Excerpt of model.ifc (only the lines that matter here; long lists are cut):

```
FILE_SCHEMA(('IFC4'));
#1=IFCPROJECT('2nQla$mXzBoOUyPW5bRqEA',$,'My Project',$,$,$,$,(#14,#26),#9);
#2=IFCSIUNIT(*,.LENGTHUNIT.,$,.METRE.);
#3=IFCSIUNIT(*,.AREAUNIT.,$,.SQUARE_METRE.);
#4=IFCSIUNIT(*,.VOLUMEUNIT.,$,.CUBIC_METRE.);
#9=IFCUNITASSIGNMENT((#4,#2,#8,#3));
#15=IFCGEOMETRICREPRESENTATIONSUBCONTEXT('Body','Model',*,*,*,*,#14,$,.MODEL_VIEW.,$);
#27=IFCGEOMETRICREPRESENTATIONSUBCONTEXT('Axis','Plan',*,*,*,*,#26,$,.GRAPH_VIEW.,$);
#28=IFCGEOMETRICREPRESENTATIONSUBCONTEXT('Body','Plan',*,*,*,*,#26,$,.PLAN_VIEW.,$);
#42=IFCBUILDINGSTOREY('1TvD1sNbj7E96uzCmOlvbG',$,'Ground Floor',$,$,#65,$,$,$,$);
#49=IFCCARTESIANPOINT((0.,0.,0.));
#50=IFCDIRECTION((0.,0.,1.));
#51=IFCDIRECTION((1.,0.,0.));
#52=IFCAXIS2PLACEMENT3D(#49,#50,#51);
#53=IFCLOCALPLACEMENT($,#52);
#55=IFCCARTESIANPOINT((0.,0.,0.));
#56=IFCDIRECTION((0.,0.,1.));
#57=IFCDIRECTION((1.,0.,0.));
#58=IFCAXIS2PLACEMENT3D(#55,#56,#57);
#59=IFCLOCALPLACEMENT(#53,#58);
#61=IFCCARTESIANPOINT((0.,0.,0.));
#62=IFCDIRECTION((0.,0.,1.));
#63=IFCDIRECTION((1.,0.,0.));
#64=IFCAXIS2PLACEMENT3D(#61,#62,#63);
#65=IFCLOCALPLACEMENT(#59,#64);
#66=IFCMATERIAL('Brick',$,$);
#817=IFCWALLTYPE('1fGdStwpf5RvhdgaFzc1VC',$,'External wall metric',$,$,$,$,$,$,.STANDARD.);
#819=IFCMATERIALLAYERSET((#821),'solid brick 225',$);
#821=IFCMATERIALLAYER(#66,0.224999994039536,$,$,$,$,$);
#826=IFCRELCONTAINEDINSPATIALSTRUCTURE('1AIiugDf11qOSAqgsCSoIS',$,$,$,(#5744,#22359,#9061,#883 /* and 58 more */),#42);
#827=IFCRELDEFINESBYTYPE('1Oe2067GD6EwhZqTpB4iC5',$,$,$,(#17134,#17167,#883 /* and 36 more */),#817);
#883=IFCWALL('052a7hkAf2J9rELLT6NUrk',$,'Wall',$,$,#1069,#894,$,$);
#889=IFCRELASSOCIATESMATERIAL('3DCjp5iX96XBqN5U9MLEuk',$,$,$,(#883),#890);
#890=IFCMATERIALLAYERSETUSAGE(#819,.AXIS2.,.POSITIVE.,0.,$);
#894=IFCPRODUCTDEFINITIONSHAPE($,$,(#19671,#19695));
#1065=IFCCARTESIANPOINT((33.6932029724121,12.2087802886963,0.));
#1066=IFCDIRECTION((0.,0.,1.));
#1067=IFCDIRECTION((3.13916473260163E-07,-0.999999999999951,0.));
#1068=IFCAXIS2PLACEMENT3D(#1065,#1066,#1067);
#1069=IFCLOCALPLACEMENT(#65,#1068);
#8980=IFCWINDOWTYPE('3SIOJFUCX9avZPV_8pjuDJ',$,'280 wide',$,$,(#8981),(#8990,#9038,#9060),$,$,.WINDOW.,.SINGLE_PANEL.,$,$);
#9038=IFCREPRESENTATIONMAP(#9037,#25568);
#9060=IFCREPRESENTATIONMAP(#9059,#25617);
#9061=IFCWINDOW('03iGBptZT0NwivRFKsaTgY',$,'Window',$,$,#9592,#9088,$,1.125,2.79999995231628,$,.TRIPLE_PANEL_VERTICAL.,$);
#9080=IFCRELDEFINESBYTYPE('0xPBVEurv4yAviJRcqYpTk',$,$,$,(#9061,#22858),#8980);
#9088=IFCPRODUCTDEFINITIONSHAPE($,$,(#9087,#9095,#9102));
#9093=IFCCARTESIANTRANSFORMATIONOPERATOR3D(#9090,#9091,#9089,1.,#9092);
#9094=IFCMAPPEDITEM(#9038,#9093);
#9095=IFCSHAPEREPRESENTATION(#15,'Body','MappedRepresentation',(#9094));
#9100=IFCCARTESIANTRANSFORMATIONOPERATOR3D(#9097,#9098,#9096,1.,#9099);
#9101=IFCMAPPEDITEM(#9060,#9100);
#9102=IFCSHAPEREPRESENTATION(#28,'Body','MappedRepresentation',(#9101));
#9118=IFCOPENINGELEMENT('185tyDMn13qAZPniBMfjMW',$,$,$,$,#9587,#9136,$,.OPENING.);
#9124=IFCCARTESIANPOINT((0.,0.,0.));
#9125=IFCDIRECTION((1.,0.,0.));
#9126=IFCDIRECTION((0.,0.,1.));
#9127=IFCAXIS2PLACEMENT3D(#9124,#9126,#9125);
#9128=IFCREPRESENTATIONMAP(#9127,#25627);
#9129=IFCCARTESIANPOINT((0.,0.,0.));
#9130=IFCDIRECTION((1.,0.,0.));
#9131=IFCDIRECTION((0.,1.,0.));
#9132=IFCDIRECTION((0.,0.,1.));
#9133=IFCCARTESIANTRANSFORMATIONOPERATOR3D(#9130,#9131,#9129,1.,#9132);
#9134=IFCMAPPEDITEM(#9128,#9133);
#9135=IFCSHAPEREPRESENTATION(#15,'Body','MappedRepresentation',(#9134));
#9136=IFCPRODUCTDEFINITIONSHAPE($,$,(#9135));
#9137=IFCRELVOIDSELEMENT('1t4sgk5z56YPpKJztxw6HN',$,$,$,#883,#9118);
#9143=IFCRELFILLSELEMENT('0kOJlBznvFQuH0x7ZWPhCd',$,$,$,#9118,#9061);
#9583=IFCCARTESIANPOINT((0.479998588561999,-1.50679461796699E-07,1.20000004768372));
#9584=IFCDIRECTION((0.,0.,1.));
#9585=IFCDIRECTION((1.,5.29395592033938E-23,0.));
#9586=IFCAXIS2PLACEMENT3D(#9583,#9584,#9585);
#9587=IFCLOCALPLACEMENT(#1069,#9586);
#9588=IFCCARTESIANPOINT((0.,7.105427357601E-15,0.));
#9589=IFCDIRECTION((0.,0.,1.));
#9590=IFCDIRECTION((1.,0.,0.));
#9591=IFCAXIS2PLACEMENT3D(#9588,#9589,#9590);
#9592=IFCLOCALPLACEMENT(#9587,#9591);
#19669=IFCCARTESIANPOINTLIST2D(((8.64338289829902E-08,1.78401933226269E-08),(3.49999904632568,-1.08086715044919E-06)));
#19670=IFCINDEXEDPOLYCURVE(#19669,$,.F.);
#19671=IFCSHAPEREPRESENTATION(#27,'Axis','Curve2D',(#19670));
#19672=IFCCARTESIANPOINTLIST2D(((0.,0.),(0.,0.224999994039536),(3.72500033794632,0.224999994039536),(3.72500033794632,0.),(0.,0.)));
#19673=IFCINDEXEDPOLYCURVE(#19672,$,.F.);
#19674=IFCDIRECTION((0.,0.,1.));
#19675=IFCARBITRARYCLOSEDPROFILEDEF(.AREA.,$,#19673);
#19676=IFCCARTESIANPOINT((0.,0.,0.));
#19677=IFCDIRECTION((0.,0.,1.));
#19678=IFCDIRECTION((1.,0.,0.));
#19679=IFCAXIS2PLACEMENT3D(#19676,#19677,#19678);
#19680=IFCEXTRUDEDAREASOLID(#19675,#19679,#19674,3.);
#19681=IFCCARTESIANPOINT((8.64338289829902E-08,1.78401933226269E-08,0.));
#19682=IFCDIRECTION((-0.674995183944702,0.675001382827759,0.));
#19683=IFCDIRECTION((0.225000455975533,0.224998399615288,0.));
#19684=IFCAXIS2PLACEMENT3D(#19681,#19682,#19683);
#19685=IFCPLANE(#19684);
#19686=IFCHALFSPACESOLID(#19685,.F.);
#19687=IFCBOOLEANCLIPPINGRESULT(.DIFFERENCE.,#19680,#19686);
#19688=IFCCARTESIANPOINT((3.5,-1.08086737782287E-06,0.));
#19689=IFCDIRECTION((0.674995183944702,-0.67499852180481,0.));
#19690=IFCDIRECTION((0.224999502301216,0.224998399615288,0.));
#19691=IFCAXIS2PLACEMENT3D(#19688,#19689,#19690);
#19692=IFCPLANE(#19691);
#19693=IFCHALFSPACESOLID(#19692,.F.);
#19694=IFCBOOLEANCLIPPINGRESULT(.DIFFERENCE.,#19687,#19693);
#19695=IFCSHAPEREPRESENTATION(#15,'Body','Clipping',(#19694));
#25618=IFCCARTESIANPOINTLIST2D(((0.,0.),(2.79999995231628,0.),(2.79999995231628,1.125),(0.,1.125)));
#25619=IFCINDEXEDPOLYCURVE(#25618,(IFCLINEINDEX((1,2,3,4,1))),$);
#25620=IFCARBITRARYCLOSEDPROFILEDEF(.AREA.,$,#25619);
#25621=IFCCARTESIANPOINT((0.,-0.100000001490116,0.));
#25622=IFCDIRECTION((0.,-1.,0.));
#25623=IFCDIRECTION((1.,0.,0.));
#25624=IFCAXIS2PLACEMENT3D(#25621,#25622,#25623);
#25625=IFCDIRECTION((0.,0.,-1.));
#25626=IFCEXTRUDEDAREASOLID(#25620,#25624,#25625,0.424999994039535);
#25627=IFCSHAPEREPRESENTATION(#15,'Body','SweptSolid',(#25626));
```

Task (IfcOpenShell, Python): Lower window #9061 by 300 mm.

```python
import numpy as np
import ifcopenshell
import ifcopenshell.api.geometry
import ifcopenshell.util.placement
import ifcopenshell.util.unit

model = ifcopenshell.open("model.ifc")
unit_scale = ifcopenshell.util.unit.calculate_unit_scale(model)

window = model.by_id(9061)
opening = window.FillsVoids[0].RelatingOpeningElement
dz = -0.3

shift = np.array([0.0, 0.0, dz])
# The window is placed relative to its opening, so it follows when the opening moves.
matrix = ifcopenshell.util.placement.get_local_placement(opening.ObjectPlacement)
matrix[:3, 3] += shift
ifcopenshell.api.geometry.edit_object_placement(
    model, product=opening, matrix=matrix, is_si=False, should_transform_children=True
)

print(f"moved by {dz * unit_scale:+.3f} m")

model.write("model_edited.ifc")
```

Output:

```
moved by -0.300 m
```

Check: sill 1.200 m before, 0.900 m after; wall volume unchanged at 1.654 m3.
